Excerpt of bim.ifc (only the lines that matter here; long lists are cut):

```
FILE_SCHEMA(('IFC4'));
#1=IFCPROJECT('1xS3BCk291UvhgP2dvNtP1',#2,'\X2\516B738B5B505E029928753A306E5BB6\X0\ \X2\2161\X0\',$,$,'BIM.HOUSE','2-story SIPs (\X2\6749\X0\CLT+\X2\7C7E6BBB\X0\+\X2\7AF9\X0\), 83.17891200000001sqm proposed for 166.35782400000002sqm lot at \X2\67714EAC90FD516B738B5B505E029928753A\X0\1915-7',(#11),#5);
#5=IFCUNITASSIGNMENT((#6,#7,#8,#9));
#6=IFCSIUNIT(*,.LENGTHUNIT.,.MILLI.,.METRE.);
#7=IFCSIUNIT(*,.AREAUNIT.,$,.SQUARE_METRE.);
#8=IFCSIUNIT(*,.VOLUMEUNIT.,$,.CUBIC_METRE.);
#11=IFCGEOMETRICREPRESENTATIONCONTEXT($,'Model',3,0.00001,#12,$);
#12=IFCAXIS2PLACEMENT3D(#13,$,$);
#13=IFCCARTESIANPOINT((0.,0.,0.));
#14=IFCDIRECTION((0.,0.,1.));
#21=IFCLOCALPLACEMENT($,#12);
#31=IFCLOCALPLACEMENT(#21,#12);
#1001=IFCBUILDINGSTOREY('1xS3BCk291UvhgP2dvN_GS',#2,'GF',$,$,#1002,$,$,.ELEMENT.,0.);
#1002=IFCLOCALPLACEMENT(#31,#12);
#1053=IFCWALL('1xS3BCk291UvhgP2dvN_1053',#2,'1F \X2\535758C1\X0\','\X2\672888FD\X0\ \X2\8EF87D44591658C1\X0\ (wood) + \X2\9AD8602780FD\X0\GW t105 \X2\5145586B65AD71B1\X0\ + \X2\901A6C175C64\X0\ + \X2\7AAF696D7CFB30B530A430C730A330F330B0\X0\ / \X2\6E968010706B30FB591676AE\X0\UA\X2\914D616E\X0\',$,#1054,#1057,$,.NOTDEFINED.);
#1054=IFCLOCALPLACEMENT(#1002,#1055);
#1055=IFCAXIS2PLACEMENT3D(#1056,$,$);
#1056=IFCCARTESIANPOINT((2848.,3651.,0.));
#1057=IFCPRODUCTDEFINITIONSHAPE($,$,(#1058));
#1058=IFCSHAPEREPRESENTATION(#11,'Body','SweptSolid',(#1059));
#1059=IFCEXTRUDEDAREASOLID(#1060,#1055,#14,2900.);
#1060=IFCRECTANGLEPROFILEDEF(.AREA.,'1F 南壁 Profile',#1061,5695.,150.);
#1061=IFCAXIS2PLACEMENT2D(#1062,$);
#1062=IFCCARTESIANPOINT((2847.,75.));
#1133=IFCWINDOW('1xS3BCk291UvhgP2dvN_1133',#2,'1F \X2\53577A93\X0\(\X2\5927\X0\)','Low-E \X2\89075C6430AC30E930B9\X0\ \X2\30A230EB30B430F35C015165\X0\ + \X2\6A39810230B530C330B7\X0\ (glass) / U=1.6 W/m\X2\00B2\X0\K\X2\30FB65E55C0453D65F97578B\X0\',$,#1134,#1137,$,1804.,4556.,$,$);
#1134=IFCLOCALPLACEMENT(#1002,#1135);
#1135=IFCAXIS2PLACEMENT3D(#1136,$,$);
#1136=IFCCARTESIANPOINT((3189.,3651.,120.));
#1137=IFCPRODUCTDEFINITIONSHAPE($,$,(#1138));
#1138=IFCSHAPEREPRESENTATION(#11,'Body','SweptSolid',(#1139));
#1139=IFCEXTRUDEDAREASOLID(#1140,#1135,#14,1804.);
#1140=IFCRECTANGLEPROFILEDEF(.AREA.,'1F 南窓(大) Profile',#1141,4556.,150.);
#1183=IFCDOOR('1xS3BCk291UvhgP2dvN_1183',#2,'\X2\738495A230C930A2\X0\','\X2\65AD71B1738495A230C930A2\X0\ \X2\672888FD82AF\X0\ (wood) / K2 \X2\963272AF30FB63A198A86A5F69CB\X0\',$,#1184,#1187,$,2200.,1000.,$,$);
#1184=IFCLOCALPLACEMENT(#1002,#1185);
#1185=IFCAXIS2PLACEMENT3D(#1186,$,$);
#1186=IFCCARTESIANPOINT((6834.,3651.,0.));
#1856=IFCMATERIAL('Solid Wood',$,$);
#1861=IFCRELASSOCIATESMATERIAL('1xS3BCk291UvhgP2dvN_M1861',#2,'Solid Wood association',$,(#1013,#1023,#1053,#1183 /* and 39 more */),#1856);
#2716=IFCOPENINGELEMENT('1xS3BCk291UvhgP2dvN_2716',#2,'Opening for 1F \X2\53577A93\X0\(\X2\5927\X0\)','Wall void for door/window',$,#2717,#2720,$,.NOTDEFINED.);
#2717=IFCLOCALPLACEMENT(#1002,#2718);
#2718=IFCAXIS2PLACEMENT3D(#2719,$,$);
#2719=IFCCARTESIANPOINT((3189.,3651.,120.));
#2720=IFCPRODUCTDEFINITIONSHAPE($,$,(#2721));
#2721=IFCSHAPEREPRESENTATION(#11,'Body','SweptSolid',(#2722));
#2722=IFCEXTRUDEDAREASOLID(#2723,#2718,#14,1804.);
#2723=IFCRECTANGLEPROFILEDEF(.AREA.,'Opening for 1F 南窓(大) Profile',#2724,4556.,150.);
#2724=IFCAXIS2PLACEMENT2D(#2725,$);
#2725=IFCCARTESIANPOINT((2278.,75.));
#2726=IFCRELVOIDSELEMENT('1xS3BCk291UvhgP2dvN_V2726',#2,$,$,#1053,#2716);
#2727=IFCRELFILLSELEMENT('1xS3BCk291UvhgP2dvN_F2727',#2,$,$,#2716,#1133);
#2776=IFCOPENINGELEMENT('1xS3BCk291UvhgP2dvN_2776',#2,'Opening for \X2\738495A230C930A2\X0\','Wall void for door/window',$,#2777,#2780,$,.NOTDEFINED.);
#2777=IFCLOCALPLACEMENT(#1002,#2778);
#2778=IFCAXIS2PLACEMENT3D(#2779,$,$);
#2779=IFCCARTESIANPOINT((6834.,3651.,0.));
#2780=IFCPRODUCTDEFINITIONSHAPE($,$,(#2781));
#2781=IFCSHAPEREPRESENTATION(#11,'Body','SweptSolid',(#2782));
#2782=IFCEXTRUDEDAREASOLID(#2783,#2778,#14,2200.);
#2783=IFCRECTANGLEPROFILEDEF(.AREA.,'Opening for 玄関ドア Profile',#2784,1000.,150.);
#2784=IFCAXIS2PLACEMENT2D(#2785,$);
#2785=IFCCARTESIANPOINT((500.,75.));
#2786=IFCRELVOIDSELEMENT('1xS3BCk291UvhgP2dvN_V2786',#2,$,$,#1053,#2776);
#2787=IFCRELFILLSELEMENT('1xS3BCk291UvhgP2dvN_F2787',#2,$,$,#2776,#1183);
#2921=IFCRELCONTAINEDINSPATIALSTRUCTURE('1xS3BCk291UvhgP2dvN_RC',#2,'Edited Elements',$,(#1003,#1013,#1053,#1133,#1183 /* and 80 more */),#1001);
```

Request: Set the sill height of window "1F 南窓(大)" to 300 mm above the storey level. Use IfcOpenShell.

```python
import numpy as np
import ifcopenshell
import ifcopenshell.api.geometry
import ifcopenshell.geom
import ifcopenshell.util.element
import ifcopenshell.util.placement
import ifcopenshell.util.shape
import ifcopenshell.util.unit

model = ifcopenshell.open("bim.ifc")
unit_scale = ifcopenshell.util.unit.calculate_unit_scale(model)

window = model.by_guid("1xS3BCk291UvhgP2dvN_1133")
opening = window.FillsVoids[0].RelatingOpeningElement
storey = ifcopenshell.util.element.get_container(window, ifc_class="IfcBuildingStorey")
level = ifcopenshell.util.placement.get_local_placement(storey.ObjectPlacement)[2, 3]

# The opening's origin need not be at the sill, so measure its lowest point.
shape = ifcopenshell.geom.create_shape(ifcopenshell.geom.settings(), opening)
bottom = ifcopenshell.util.shape.get_shape_bottom_elevation(shape, shape.geometry) / unit_scale
dz = level + 300.0 - bottom

shift = np.array([0.0, 0.0, dz])
# The window is not placed relative to its opening, so move both.
for product in (opening, window):
    matrix = ifcopenshell.util.placement.get_local_placement(product.ObjectPlacement)
    matrix[:3, 3] += shift
    ifcopenshell.api.geometry.edit_object_placement(model, product=product, matrix=matrix, is_si=False)

print(f"moved by {dz * unit_scale:+.3f} m")

model.write("bim_edited.ifc")
```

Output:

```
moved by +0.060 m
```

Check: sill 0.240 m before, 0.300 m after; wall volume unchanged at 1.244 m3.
